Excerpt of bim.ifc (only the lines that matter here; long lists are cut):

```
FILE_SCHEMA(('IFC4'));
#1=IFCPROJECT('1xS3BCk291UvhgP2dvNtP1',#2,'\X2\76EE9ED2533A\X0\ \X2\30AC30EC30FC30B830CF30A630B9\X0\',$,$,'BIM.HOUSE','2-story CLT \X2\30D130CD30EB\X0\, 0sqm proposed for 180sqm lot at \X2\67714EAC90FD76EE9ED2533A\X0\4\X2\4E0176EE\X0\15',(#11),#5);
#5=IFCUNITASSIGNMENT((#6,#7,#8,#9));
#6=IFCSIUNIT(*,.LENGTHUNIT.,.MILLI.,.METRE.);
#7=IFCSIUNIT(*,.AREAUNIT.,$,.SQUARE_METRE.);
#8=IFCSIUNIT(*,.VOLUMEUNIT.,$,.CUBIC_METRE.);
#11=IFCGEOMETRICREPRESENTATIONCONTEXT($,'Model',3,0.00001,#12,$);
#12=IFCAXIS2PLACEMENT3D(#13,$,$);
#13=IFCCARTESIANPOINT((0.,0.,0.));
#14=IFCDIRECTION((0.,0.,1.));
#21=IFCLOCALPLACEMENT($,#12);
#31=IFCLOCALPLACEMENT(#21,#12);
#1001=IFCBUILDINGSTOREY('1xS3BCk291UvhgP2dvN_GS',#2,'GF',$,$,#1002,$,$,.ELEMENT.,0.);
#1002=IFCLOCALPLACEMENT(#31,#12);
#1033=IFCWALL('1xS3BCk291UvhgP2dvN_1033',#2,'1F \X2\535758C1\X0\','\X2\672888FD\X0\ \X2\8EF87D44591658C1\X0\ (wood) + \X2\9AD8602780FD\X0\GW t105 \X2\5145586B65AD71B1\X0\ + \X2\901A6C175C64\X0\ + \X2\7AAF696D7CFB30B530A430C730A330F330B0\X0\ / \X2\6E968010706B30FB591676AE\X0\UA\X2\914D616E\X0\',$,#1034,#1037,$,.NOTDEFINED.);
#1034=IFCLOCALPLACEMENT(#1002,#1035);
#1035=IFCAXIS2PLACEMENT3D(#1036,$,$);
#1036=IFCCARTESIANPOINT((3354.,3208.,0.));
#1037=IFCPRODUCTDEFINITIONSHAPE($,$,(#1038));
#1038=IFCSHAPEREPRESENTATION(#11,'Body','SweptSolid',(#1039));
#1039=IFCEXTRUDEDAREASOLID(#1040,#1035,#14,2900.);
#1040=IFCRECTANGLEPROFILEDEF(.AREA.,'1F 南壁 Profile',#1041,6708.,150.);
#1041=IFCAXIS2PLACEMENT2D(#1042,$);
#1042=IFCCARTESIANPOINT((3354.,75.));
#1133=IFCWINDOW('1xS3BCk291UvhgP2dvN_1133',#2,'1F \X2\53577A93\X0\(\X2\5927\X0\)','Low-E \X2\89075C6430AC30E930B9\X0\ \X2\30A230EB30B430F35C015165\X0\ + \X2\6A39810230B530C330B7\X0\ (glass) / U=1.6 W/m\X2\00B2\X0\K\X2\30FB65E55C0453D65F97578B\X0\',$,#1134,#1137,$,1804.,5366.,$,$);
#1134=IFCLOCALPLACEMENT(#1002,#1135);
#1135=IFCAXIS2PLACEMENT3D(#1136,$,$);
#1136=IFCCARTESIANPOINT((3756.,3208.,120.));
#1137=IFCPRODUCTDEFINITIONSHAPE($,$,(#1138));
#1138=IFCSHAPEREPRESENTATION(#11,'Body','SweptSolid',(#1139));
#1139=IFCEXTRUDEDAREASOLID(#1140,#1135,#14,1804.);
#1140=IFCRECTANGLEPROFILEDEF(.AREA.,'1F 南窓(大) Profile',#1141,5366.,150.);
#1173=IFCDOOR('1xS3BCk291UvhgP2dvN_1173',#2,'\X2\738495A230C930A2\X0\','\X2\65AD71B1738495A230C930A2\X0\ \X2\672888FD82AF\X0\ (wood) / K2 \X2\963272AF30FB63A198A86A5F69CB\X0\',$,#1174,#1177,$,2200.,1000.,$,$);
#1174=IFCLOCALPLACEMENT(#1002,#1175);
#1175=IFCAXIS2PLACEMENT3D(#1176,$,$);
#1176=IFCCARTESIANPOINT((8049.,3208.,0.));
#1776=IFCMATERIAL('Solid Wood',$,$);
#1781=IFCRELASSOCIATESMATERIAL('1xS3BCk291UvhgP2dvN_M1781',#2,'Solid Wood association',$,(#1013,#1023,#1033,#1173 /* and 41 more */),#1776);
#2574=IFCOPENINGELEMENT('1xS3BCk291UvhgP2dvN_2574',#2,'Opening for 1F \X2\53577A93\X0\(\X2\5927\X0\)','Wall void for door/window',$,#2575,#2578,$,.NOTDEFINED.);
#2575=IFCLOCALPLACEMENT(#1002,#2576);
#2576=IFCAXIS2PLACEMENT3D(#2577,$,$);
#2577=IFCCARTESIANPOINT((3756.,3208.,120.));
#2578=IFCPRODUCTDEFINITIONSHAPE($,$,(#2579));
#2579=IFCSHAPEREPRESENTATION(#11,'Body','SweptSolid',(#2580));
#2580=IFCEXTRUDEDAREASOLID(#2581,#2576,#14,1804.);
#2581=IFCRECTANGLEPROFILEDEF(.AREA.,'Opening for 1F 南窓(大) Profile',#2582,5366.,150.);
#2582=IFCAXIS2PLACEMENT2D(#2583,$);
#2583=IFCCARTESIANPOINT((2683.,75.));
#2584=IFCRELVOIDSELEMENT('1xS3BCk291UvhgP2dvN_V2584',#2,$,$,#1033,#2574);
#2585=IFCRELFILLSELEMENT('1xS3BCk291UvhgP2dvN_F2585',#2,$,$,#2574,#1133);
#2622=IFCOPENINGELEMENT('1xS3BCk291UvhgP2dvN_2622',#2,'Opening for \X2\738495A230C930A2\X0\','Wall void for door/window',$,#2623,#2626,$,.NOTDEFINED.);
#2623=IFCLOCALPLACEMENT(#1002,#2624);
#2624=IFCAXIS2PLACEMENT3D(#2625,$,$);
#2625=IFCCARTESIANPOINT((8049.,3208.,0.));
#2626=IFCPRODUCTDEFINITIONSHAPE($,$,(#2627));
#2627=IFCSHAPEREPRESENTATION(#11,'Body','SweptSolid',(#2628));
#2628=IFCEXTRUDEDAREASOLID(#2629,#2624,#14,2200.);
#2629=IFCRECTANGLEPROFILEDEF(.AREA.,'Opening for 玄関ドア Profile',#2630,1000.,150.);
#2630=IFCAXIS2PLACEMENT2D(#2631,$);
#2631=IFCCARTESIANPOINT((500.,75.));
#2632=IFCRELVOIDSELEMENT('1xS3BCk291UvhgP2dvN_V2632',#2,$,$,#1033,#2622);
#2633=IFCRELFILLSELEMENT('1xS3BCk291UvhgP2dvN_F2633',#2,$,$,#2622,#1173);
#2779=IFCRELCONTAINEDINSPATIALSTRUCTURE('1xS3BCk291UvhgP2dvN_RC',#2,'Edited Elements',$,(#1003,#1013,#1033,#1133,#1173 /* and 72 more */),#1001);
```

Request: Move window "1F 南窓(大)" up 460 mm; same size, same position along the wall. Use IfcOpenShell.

```python
import numpy as np
import ifcopenshell
import ifcopenshell.api.geometry
import ifcopenshell.util.placement
import ifcopenshell.util.unit

model = ifcopenshell.open("bim.ifc")
unit_scale = ifcopenshell.util.unit.calculate_unit_scale(model)

window = model.by_guid("1xS3BCk291UvhgP2dvN_1133")
opening = window.FillsVoids[0].RelatingOpeningElement
dz = 460.0

shift = np.array([0.0, 0.0, dz])
# The window is not placed relative to its opening, so move both.
for product in (opening, window):
    matrix = ifcopenshell.util.placement.get_local_placement(product.ObjectPlacement)
    matrix[:3, 3] += shift
    ifcopenshell.api.geometry.edit_object_placement(model, product=product, matrix=matrix, is_si=False)

print(f"moved by {dz * unit_scale:+.3f} m")

model.write("bim_edited.ifc")
```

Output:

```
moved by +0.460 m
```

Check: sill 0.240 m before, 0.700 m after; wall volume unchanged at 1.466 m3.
